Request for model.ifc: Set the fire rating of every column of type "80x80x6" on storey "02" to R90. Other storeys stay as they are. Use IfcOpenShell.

First a look at what the model holds.

```python
import ifcopenshell
import ifcopenshell.util.element

model = ifcopenshell.open("model.ifc")
print(model.schema)
storey = next(s for s in model.by_type("IfcBuildingStorey") if s.Name == "02")
columns = [e for e in ifcopenshell.util.element.get_decomposition(storey) if e.is_a("IfcColumn")]
seen = {}
for e in columns:
    element_type = ifcopenshell.util.element.get_type(e)
    key = (element_type.Name if element_type != e and element_type else None, ifcopenshell.util.element.get_pset(e, "Pset_ColumnCommon", "FireRating"))
    seen[key] = seen.get(key, 0) + 1
for (name, value), count in sorted(seen.items(), key=str):
    print(count, "x", name, "|", value)
```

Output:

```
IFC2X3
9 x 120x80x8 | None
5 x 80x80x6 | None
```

```python
import ifcopenshell
import ifcopenshell.api.pset
import ifcopenshell.util.element

model = ifcopenshell.open("model.ifc")

storey = next(s for s in model.by_type("IfcBuildingStorey") if s.Name == "02")
columns = [e for e in ifcopenshell.util.element.get_decomposition(storey) if e.is_a("IfcColumn")]

count = 0
for e in columns:
    element_type = ifcopenshell.util.element.get_type(e)
    if element_type in (None, e) or element_type.Name != "80x80x6":
        continue
    # add_pset returns the element's existing set when there is one.
    pset = ifcopenshell.api.pset.add_pset(model, product=e, name="Pset_ColumnCommon")
    ifcopenshell.api.pset.edit_pset(model, pset=pset, properties={"FireRating": "R90"})
    count += 1

print(count, "columns updated")

model.write("model_updated.ifc")
```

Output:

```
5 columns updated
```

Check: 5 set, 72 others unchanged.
